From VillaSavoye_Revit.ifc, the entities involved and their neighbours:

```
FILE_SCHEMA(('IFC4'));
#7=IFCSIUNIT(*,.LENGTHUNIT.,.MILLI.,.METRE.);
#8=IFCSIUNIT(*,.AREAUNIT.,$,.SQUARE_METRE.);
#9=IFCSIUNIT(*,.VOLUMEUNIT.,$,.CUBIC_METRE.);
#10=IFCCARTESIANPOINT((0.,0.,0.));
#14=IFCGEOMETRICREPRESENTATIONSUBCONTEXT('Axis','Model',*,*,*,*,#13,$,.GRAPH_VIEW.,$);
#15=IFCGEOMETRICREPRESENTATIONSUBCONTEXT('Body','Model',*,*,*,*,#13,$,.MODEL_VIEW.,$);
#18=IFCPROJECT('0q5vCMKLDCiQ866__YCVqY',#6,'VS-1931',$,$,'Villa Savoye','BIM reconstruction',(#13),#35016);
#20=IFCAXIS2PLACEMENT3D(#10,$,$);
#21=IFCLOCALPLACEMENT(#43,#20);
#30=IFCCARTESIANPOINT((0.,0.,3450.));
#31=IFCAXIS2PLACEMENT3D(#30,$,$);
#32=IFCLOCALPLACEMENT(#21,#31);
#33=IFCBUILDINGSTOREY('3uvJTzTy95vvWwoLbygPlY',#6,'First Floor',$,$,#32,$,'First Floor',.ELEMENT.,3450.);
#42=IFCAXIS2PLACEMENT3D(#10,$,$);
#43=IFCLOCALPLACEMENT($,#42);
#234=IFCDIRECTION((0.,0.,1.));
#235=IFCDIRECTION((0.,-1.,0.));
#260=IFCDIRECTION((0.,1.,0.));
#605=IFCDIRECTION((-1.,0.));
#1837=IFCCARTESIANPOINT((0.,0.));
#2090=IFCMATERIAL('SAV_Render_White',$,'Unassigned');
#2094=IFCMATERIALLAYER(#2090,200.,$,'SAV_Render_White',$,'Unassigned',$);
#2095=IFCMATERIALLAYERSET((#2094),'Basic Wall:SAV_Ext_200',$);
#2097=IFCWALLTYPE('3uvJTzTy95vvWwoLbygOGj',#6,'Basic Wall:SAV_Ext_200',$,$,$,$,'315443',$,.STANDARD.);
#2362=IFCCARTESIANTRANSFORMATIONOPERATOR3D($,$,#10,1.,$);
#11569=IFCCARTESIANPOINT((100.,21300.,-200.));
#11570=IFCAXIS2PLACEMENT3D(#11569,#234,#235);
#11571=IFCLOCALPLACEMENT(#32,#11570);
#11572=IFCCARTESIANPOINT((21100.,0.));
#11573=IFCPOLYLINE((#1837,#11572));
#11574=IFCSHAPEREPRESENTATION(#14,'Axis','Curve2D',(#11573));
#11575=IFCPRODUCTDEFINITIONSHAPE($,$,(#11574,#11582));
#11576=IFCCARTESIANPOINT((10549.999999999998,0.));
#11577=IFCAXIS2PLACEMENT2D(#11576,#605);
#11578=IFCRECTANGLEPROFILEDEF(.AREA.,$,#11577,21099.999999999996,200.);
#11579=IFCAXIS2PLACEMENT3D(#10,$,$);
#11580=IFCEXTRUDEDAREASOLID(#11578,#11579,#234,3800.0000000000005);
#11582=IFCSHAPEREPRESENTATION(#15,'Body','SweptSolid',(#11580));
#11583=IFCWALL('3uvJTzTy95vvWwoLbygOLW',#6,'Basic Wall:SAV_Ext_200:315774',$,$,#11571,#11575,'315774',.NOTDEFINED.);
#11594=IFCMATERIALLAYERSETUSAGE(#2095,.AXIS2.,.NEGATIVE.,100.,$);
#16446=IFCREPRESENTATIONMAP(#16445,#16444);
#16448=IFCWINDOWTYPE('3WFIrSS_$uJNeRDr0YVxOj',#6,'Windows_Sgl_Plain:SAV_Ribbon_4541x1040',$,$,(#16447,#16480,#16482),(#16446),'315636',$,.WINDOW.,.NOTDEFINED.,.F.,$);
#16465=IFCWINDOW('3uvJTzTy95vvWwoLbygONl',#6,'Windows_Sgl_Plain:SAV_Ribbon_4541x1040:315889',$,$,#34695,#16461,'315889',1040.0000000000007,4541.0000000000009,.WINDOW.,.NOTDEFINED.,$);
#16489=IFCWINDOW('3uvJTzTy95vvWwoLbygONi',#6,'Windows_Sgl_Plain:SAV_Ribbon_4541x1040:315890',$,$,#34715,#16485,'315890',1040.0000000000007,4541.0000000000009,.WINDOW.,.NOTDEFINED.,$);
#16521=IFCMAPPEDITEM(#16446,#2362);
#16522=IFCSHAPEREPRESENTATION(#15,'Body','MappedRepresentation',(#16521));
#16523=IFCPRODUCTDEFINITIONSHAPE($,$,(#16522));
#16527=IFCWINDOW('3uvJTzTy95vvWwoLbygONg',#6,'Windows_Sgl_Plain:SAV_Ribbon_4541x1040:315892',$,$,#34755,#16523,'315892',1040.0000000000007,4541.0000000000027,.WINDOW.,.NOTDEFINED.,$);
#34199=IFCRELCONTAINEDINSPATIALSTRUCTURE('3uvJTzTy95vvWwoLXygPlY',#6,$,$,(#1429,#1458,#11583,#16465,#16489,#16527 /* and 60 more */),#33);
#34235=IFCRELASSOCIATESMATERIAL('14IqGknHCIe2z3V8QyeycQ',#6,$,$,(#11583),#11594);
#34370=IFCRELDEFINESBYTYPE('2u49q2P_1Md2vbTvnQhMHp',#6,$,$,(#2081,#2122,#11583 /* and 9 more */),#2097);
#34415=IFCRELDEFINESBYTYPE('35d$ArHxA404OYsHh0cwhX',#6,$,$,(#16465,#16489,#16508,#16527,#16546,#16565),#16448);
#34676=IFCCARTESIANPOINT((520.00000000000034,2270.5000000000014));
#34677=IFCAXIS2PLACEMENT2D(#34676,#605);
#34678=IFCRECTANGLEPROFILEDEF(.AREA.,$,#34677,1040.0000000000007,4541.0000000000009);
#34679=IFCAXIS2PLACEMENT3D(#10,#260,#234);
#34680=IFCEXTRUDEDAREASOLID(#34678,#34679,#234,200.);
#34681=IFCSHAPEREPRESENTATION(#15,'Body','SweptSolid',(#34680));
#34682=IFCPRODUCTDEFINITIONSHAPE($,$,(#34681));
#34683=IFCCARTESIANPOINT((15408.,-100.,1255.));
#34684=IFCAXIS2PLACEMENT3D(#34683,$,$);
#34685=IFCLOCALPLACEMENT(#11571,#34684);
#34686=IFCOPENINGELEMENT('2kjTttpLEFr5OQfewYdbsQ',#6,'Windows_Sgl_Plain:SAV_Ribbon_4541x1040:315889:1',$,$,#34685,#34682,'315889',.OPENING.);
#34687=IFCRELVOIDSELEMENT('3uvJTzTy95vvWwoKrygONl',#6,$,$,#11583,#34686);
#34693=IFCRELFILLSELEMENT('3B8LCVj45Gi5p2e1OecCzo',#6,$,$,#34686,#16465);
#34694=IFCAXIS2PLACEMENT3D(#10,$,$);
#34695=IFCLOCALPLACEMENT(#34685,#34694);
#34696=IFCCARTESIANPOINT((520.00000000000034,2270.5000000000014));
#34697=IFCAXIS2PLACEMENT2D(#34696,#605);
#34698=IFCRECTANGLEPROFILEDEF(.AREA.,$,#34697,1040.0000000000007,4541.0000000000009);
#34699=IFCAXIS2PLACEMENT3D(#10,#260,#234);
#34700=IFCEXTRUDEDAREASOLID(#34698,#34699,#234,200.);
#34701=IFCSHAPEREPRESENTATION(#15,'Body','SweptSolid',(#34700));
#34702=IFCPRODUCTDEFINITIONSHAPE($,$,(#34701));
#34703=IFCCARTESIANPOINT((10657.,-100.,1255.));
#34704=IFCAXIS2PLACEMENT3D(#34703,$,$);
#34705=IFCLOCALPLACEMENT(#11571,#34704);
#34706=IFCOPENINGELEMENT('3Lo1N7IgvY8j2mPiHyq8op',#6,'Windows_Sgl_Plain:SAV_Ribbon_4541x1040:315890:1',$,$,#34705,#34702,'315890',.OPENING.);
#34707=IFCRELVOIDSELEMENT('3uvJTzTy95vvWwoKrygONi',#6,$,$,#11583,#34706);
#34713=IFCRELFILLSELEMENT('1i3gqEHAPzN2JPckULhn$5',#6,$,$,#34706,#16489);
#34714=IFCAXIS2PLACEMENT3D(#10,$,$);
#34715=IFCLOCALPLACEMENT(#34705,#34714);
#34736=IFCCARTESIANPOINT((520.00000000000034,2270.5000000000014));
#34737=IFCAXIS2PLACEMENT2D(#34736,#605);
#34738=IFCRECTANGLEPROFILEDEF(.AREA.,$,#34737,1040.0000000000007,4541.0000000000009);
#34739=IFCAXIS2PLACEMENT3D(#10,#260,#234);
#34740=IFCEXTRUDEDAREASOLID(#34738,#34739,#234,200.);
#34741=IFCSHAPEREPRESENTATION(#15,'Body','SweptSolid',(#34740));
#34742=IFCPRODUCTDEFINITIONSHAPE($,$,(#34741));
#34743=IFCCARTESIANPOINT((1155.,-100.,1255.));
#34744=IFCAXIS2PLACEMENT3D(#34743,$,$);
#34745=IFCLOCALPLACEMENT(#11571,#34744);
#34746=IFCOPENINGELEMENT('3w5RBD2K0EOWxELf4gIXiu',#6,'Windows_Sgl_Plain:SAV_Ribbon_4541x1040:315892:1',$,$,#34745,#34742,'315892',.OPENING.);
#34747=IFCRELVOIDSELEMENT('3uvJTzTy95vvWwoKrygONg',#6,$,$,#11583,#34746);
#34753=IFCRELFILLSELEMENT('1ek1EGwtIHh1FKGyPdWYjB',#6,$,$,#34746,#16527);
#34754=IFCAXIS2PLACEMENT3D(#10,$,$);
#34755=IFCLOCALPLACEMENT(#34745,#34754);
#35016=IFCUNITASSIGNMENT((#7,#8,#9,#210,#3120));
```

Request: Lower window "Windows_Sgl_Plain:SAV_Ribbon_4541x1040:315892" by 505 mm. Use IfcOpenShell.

```python
import numpy as np
import ifcopenshell
import ifcopenshell.api.geometry
import ifcopenshell.util.placement
import ifcopenshell.util.unit

model = ifcopenshell.open("VillaSavoye_Revit.ifc")
unit_scale = ifcopenshell.util.unit.calculate_unit_scale(model)

window = model.by_guid("3uvJTzTy95vvWwoLbygONg")
opening = window.FillsVoids[0].RelatingOpeningElement
dz = -505.0

shift = np.array([0.0, 0.0, dz])
# The window is placed relative to its opening, so it follows when the opening moves.
matrix = ifcopenshell.util.placement.get_local_placement(opening.ObjectPlacement)
matrix[:3, 3] += shift
ifcopenshell.api.geometry.edit_object_placement(
    model, product=opening, matrix=matrix, is_si=False, should_transform_children=True
)

print(f"moved by {dz * unit_scale:+.3f} m")

model.write("VillaSavoye_Revit_edited.ifc")
```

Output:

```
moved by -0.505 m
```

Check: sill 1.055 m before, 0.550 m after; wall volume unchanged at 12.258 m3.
